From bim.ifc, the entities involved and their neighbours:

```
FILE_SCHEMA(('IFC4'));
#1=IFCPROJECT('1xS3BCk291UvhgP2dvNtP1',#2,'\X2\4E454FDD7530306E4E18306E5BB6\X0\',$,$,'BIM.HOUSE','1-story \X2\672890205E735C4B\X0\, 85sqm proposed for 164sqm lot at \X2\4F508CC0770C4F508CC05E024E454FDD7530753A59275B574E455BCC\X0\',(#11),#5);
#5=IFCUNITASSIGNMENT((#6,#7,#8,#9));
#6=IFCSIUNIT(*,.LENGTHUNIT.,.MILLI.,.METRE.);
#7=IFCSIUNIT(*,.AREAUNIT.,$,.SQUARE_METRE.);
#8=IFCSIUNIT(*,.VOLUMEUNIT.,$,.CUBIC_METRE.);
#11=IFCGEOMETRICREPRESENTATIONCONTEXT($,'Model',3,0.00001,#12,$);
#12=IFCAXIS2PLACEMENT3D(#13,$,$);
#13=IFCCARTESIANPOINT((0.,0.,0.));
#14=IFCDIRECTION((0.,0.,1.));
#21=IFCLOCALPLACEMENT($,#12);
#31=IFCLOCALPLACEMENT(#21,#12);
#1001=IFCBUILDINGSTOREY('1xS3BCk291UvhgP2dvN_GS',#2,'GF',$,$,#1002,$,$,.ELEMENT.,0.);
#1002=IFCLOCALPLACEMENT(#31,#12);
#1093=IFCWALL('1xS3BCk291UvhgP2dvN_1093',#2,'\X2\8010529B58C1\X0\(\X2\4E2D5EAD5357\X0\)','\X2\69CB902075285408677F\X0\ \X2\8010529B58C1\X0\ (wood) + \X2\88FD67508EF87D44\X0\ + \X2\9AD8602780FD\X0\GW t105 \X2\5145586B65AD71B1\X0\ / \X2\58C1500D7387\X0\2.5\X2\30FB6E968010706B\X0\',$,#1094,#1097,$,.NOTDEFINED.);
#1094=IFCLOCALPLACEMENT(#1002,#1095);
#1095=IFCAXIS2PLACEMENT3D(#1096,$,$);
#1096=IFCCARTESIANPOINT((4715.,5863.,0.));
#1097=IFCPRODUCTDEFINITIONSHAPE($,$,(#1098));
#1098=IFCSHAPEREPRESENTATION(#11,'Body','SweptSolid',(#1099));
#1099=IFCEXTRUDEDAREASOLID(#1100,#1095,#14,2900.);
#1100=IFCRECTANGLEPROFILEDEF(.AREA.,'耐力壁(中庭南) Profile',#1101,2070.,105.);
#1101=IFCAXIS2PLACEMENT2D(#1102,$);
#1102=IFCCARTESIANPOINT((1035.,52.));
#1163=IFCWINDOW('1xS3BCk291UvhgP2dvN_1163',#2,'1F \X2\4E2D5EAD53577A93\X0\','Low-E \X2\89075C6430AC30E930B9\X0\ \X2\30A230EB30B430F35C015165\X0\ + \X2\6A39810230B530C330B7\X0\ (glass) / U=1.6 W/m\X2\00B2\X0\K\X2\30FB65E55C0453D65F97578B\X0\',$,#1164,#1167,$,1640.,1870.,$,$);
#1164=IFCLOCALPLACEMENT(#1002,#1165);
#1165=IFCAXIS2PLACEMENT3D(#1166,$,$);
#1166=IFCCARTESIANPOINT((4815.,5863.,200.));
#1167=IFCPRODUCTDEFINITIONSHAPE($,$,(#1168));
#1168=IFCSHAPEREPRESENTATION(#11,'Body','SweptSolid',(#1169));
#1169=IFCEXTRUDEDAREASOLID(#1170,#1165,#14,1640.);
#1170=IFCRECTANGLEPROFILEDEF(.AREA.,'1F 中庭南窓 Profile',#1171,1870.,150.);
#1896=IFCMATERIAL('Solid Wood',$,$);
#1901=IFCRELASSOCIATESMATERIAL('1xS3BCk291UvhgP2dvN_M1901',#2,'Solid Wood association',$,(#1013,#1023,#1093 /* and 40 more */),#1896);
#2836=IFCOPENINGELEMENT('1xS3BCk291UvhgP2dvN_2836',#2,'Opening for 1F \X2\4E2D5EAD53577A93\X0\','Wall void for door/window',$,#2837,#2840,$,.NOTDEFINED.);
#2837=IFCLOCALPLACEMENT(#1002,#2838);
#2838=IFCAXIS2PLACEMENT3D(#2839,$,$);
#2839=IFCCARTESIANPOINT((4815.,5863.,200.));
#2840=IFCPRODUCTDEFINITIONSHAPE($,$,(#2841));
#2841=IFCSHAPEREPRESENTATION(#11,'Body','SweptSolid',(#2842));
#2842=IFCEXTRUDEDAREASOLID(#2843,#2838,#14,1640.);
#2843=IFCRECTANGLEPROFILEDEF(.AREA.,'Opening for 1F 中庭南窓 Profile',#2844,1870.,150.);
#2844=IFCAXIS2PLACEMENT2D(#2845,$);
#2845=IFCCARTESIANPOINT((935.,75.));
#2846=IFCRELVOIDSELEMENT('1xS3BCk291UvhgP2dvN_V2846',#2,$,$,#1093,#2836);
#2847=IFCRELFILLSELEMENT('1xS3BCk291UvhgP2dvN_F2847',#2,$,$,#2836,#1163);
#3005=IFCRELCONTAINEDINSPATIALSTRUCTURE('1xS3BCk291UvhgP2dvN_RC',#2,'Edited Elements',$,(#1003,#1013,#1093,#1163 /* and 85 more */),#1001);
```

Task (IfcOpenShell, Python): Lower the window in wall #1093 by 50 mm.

```python
import numpy as np
import ifcopenshell
import ifcopenshell.api.geometry
import ifcopenshell.util.placement
import ifcopenshell.util.unit

model = ifcopenshell.open("bim.ifc")
unit_scale = ifcopenshell.util.unit.calculate_unit_scale(model)

window = model.by_guid("1xS3BCk291UvhgP2dvN_1163")
opening = window.FillsVoids[0].RelatingOpeningElement
dz = -0.05 / unit_scale

shift = np.array([0.0, 0.0, dz])
# The window is not placed relative to its opening, so move both.
for product in (opening, window):
    matrix = ifcopenshell.util.placement.get_local_placement(product.ObjectPlacement)
    matrix[:3, 3] += shift
    ifcopenshell.api.geometry.edit_object_placement(model, product=product, matrix=matrix, is_si=False)

print(f"moved by {dz * unit_scale:+.3f} m")

model.write("bim_edited.ifc")
```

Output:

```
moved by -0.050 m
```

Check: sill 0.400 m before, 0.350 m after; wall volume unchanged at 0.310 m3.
